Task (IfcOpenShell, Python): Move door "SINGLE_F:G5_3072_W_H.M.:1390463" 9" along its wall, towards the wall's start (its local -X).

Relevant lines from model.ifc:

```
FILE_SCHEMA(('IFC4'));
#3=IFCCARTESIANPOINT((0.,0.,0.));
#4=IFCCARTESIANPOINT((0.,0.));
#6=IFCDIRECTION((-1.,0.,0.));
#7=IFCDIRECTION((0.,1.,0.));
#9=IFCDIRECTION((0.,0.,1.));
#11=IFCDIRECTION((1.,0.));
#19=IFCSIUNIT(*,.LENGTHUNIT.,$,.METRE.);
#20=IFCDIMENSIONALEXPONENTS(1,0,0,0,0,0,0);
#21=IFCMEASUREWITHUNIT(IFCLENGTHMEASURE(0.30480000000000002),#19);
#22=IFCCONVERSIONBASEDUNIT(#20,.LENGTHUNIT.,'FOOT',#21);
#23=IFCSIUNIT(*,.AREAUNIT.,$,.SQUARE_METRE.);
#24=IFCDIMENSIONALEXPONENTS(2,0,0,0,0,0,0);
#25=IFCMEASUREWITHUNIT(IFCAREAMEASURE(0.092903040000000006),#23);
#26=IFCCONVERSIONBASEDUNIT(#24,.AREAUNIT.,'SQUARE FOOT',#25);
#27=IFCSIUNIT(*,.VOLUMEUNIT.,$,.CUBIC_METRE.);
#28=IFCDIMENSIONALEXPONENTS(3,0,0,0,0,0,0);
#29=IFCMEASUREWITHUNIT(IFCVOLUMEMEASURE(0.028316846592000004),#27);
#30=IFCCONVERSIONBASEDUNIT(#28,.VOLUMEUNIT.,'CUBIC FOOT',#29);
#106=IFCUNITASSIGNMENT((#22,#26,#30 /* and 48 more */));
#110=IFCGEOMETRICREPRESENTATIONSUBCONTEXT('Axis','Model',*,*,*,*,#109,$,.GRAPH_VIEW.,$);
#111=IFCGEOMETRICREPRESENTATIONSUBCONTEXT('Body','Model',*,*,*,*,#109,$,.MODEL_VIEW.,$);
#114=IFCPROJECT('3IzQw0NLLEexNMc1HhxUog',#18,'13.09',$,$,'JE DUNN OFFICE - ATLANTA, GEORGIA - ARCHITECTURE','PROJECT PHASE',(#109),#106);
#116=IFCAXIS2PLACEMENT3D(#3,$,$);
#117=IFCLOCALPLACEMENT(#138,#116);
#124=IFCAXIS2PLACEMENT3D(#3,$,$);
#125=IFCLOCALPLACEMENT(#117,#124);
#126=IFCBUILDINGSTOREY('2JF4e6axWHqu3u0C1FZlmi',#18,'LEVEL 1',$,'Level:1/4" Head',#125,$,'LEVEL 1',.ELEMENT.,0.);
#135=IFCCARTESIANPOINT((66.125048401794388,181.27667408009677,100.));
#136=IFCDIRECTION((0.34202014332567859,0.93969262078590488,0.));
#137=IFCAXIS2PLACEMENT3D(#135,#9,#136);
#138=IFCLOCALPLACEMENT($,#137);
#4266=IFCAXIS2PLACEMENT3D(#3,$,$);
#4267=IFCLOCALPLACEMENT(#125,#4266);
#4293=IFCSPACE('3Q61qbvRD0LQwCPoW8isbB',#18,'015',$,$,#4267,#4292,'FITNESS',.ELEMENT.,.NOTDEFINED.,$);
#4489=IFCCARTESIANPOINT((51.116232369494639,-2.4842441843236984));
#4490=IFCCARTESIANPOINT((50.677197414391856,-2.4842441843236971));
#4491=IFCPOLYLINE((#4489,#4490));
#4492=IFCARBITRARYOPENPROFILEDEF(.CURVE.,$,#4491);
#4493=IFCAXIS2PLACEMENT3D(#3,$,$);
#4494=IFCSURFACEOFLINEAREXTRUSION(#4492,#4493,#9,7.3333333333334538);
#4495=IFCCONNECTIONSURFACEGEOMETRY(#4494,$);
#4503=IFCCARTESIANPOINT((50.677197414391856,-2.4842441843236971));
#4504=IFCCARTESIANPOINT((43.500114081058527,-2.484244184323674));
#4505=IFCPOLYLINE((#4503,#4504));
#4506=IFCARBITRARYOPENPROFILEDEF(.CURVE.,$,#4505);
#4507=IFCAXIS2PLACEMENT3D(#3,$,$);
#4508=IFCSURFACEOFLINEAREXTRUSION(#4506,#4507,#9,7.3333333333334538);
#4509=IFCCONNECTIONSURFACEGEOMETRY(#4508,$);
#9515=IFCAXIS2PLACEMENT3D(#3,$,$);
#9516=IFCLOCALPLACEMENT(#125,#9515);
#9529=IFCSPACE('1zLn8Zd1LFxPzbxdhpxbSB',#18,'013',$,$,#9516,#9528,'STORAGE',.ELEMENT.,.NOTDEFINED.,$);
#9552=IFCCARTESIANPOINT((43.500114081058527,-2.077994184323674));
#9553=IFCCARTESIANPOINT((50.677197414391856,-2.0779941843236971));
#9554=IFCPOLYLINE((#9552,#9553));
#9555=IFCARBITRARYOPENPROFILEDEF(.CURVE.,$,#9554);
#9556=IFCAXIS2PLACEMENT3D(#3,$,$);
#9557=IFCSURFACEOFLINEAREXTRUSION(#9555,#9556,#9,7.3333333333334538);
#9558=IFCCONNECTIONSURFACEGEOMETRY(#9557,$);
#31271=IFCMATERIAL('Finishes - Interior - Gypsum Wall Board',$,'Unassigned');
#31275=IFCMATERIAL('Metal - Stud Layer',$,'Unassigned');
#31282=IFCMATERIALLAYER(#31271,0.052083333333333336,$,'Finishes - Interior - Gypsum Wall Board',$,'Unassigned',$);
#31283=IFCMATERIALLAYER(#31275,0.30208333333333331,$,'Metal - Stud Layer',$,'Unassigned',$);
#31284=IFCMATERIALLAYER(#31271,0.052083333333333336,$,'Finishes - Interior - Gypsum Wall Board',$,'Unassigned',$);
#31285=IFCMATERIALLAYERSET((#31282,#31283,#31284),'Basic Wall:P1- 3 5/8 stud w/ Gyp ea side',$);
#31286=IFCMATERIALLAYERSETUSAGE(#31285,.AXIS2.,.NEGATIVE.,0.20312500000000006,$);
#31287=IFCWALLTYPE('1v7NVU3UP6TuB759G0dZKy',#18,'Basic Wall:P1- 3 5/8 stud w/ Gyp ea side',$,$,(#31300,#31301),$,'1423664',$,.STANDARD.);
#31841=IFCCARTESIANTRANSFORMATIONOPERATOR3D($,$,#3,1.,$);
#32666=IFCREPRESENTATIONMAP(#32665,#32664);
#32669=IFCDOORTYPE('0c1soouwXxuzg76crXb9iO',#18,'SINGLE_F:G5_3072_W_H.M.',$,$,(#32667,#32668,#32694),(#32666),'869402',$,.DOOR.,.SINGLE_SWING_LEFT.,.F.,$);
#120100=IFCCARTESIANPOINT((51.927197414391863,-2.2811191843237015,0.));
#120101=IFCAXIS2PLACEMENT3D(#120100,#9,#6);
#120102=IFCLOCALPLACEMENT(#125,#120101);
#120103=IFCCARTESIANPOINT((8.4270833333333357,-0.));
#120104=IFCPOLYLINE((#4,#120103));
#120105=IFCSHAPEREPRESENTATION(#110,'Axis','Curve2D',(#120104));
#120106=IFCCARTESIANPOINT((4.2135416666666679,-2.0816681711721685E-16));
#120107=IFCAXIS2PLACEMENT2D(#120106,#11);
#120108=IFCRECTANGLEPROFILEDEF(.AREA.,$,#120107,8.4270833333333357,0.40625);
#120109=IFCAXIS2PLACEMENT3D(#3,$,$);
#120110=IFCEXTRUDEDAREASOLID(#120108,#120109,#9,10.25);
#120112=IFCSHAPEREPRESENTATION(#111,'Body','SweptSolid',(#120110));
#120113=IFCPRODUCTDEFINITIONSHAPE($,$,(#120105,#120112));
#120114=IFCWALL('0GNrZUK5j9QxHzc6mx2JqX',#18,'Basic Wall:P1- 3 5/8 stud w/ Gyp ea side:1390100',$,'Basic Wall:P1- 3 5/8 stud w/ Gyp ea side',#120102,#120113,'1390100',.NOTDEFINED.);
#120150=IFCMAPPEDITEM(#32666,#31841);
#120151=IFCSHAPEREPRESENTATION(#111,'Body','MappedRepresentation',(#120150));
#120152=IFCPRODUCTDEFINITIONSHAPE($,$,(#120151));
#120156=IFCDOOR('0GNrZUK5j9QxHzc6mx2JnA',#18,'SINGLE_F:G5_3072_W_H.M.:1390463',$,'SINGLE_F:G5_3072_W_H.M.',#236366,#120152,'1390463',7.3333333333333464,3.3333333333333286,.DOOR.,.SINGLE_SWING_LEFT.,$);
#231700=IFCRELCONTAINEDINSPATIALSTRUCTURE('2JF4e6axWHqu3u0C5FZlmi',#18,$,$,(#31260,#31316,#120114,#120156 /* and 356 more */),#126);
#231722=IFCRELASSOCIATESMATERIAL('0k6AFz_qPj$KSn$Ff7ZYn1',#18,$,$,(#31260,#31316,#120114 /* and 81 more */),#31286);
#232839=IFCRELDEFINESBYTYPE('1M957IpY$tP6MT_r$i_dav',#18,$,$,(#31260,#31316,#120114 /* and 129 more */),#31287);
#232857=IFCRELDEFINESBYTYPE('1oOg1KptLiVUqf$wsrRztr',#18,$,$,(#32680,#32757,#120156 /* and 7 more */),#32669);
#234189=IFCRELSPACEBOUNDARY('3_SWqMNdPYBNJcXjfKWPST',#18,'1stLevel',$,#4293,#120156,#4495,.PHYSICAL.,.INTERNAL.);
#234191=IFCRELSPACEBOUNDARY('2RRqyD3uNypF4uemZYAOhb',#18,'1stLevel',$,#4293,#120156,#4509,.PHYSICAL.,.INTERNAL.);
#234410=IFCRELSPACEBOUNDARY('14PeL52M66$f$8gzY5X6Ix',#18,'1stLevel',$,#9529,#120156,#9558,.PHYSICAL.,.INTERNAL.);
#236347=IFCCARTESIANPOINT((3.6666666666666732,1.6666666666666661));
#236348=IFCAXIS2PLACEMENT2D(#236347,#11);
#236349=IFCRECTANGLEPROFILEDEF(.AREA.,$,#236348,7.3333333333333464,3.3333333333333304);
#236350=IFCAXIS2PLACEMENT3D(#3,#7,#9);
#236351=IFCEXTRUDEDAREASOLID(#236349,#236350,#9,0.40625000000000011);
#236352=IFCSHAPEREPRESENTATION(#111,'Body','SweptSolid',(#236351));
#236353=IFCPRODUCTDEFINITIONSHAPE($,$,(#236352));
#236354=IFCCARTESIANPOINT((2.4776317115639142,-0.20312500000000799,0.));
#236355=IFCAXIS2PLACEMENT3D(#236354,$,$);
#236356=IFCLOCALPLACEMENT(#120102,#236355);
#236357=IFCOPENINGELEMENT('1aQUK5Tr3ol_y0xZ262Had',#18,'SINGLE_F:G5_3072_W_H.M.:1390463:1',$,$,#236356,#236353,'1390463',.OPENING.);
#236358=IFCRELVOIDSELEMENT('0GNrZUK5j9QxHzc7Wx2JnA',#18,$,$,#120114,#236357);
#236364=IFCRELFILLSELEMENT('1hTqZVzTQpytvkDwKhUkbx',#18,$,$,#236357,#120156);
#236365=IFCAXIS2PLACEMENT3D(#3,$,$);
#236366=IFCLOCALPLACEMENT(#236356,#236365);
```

```python
import numpy as np
import ifcopenshell
import ifcopenshell.api.geometry
import ifcopenshell.util.placement
import ifcopenshell.util.unit

model = ifcopenshell.open("model.ifc")
unit_scale = ifcopenshell.util.unit.calculate_unit_scale(model)

door = model.by_id(120156)
opening = door.FillsVoids[0].RelatingOpeningElement
wall = opening.VoidsElements[0].RelatingBuildingElement

wall_matrix = ifcopenshell.util.placement.get_local_placement(wall.ObjectPlacement)
shift = wall_matrix[:3, 0] * -9 * 0.0254 / unit_scale
before = ifcopenshell.util.placement.get_local_placement(door.ObjectPlacement)[:3, 3].copy()

# The door is placed relative to its opening, so it follows when the opening moves.
matrix = ifcopenshell.util.placement.get_local_placement(opening.ObjectPlacement)
matrix[:3, 3] += shift
ifcopenshell.api.geometry.edit_object_placement(
    model, product=opening, matrix=matrix, is_si=False, should_transform_children=True
)

# Space boundary surfaces are stored in each space's coordinates; move them too.
for rel in door.ProvidesBoundaries:
    if not rel.ConnectionGeometry:
        continue
    surface = rel.ConnectionGeometry.SurfaceOnRelatingElement
    space_matrix = ifcopenshell.util.placement.get_local_placement(rel.RelatingSpace.ObjectPlacement)
    point = np.array(surface.Position.Location.Coordinates) + space_matrix[:3, :3].T @ shift
    surface.Position = model.createIfcAxis2Placement3D(
        model.createIfcCartesianPoint(point.tolist()), surface.Position.Axis, surface.Position.RefDirection
    )

after = ifcopenshell.util.placement.get_local_placement(door.ObjectPlacement)[:3, 3]
print("door moved by", (after - before).round(3) + 0.0)

model.write("model_rev.ifc")
```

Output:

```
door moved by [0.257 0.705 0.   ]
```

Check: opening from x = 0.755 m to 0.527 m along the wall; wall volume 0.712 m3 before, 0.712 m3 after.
